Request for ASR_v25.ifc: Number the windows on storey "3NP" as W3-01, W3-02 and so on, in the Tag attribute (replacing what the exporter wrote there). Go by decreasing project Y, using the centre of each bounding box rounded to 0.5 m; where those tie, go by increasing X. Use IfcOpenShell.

First a look at what the model holds.

```python
import ifcopenshell
import ifcopenshell.util.element
import ifcopenshell.util.placement

model = ifcopenshell.open("ASR_v25.ifc")
print(model.schema)
storey = next(s for s in model.by_type("IfcBuildingStorey") if s.Name == "3NP")
windows = [e for e in ifcopenshell.util.element.get_decomposition(storey) if e.is_a("IfcWindow")]
for e in sorted(windows, key=lambda e: e.id()):
    origin = ifcopenshell.util.placement.get_local_placement(e.ObjectPlacement)[:3, 3]
    print(e.id(), e.Tag, e.Name, origin.round(2) + 0.0, sep=" | ")
```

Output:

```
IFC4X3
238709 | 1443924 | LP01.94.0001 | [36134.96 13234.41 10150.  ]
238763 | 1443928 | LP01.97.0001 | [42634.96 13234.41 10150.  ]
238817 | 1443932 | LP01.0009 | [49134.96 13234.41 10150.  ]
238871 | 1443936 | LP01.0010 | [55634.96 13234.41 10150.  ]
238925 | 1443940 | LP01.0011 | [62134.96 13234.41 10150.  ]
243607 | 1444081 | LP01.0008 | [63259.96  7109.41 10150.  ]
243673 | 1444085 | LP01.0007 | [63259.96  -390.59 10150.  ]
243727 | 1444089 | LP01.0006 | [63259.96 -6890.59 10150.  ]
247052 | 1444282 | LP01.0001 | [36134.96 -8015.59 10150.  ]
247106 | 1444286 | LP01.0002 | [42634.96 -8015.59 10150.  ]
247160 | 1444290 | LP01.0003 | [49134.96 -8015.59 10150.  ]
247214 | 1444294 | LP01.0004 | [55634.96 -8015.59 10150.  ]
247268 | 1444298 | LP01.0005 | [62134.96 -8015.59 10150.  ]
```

```python
import ifcopenshell
import ifcopenshell.geom
import ifcopenshell.util.element
import ifcopenshell.util.shape

model = ifcopenshell.open("ASR_v25.ifc")
settings = ifcopenshell.geom.settings()
settings.set("use-world-coords", True)


def centre(element):
    shape = ifcopenshell.geom.create_shape(settings, element)
    return ifcopenshell.util.shape.get_bbox_centroid(shape.geometry)


storey = next(s for s in model.by_type("IfcBuildingStorey") if s.Name == "3NP")
windows = [e for e in ifcopenshell.util.element.get_decomposition(storey) if e.is_a("IfcWindow")]

# Insertion points can sit at a corner or the storey origin, so sort by the geometry (in metres).
centres = {e: centre(e) for e in windows}
windows.sort(key=lambda e: (-round(centres[e][1] / 0.5), centres[e][0]))

for i, e in enumerate(windows, start=1):
    number = f"W3-{i:02d}"
    e.Tag = number
    print(e.id(), number)

model.write("ASR_v25_rev.ifc")
```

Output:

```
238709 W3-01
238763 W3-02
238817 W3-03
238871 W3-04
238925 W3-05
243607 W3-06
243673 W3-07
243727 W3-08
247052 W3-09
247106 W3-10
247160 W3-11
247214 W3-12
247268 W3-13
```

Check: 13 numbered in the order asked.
